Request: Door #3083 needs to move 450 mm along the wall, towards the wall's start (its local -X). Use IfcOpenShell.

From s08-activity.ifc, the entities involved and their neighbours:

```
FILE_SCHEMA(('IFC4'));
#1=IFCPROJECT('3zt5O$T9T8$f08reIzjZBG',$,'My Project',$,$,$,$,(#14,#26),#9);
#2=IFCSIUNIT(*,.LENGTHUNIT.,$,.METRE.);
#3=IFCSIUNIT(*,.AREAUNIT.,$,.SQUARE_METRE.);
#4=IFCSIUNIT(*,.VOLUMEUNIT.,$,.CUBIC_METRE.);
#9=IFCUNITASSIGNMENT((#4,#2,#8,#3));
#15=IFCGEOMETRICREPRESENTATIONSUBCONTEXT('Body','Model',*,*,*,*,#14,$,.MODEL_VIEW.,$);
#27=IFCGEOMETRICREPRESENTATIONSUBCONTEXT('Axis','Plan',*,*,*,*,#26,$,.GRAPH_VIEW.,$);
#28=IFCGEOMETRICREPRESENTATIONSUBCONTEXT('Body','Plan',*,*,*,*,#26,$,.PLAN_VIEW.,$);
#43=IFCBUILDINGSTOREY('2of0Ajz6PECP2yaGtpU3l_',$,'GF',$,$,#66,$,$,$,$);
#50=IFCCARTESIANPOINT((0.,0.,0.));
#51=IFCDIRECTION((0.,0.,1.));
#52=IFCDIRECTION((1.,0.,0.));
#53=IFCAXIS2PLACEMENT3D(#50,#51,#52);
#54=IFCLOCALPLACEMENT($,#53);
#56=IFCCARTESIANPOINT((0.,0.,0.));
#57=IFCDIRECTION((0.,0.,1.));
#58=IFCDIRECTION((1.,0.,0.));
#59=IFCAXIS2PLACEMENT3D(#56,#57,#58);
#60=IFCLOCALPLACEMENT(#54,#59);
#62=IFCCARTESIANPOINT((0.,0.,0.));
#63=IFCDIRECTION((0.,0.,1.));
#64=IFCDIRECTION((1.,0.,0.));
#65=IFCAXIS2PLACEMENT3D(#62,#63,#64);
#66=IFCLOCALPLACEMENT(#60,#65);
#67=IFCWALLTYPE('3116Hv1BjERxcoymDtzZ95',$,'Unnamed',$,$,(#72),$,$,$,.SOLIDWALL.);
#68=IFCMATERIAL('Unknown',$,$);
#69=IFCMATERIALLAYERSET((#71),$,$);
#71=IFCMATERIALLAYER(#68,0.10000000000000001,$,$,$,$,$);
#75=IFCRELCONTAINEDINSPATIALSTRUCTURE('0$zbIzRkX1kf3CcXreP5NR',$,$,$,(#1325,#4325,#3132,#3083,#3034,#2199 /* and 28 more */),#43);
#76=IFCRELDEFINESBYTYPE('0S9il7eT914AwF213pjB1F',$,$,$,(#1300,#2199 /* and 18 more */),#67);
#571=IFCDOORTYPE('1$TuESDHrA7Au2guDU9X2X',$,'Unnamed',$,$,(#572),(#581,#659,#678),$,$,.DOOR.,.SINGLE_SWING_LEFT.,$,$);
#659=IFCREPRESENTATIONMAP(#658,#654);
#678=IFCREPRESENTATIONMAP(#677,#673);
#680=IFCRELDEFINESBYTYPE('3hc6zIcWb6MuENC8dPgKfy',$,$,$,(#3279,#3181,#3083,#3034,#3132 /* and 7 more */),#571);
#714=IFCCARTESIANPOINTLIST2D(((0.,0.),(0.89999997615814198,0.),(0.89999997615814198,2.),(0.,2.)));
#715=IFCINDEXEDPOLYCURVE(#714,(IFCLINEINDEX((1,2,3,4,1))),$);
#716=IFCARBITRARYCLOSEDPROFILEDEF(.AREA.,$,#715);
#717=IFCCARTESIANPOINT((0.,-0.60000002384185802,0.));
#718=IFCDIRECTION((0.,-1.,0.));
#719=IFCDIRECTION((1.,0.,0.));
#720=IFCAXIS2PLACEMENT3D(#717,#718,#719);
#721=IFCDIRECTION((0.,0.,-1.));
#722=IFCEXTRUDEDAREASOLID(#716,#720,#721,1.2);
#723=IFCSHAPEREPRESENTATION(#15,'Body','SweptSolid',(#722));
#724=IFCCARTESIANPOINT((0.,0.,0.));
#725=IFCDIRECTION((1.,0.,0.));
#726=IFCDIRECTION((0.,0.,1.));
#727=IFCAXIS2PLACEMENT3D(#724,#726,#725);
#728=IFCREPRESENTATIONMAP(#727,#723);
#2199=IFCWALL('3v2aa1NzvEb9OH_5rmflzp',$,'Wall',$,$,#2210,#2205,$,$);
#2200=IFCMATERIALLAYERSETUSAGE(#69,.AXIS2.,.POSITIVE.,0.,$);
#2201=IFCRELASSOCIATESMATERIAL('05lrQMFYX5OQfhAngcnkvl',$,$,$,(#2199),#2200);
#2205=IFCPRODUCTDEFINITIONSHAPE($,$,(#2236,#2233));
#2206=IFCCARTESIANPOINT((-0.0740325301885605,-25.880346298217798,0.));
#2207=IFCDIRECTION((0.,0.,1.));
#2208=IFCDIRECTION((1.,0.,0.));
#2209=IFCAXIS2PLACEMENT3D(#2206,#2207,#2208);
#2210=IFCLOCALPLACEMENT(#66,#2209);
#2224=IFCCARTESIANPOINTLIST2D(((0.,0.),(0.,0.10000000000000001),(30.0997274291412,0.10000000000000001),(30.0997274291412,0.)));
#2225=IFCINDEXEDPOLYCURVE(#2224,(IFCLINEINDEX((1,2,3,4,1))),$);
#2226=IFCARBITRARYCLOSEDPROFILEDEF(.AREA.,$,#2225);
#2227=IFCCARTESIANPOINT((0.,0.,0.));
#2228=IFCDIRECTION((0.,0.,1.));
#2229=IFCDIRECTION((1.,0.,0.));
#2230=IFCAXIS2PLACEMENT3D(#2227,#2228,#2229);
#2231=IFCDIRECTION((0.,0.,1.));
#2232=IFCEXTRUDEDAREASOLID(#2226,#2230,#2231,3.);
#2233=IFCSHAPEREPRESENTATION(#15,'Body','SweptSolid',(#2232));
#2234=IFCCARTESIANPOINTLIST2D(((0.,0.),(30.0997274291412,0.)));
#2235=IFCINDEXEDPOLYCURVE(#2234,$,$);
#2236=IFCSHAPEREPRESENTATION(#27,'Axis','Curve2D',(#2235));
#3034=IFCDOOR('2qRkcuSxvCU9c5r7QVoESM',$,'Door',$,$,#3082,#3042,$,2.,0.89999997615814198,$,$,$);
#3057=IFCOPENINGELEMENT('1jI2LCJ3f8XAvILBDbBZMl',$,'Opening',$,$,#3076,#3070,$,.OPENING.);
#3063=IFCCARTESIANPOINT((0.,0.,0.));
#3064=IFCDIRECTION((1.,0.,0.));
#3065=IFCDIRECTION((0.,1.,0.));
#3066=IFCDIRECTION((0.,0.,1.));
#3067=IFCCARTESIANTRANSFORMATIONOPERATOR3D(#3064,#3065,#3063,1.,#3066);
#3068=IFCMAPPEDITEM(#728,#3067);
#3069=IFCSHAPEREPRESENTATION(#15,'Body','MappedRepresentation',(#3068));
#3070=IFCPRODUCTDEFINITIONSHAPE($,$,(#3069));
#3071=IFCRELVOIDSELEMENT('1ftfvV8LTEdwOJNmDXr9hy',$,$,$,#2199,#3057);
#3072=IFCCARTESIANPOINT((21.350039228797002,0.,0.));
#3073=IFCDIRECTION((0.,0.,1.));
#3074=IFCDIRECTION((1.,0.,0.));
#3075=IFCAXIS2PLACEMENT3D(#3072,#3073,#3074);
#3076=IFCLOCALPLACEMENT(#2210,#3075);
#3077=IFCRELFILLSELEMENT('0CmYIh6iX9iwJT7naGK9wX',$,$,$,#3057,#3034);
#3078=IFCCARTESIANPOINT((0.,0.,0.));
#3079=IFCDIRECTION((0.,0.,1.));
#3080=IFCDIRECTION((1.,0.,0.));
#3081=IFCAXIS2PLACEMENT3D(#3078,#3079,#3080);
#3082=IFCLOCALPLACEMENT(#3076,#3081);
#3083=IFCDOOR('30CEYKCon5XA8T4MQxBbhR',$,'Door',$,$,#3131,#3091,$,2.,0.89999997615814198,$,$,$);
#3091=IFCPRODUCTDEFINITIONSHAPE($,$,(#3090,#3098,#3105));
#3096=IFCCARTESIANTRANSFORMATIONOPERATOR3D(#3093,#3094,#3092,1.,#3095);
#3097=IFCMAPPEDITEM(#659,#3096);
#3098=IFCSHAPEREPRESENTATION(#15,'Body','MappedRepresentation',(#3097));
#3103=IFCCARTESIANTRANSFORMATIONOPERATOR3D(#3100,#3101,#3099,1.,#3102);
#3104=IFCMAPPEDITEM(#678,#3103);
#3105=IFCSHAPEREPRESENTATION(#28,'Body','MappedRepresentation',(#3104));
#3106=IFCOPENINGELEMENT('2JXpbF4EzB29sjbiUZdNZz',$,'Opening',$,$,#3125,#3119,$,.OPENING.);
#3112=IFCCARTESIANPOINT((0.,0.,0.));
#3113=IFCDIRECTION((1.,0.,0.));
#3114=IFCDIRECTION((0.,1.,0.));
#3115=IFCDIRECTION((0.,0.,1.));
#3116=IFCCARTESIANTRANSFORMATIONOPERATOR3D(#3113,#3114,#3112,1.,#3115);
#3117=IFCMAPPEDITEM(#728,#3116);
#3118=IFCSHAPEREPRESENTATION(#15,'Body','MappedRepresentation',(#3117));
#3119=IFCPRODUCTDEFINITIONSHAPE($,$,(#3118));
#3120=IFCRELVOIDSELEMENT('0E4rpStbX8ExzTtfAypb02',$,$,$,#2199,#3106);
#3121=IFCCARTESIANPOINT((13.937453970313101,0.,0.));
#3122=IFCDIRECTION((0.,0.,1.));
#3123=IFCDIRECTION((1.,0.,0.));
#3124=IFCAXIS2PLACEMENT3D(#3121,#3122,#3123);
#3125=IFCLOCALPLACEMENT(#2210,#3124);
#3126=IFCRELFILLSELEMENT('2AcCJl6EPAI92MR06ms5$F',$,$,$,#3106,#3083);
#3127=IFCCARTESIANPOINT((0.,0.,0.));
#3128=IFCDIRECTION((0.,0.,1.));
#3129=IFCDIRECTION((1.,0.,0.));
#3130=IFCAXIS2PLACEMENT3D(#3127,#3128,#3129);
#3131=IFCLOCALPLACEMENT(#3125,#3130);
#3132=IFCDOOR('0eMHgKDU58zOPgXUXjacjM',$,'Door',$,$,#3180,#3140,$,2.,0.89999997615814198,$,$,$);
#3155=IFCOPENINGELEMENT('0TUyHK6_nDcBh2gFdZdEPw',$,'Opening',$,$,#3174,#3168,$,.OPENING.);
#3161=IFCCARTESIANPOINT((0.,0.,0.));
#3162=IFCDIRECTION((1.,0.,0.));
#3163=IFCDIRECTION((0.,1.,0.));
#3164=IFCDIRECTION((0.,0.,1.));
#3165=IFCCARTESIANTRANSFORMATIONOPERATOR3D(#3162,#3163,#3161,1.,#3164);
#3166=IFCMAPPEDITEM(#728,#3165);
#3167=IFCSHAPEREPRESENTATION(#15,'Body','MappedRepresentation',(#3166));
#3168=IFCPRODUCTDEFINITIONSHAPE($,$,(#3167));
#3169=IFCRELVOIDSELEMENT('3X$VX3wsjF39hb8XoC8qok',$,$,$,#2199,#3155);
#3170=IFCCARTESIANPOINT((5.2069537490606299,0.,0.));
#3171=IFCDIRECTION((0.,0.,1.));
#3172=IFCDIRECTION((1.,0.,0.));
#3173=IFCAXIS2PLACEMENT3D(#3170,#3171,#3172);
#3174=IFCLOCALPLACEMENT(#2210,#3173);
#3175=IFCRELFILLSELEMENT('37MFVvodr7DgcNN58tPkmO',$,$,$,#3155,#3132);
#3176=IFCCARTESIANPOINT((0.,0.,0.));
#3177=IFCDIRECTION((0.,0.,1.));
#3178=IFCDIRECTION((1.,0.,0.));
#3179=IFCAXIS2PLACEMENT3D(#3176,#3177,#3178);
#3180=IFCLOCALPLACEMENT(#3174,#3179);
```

```python
import ifcopenshell
import ifcopenshell.api.geometry
import ifcopenshell.util.placement

model = ifcopenshell.open("s08-activity.ifc")

door = model.by_id(3083)
opening = door.FillsVoids[0].RelatingOpeningElement
wall = opening.VoidsElements[0].RelatingBuildingElement

wall_matrix = ifcopenshell.util.placement.get_local_placement(wall.ObjectPlacement)
shift = wall_matrix[:3, 0] * -0.45
before = ifcopenshell.util.placement.get_local_placement(door.ObjectPlacement)[:3, 3].copy()

# The door is placed relative to its opening, so it follows when the opening moves.
matrix = ifcopenshell.util.placement.get_local_placement(opening.ObjectPlacement)
matrix[:3, 3] += shift
ifcopenshell.api.geometry.edit_object_placement(
    model, product=opening, matrix=matrix, is_si=False, should_transform_children=True
)

after = ifcopenshell.util.placement.get_local_placement(door.ObjectPlacement)[:3, 3]
print("door moved by", (after - before).round(3) + 0.0)

model.write("s08-activity_updated.ifc")
```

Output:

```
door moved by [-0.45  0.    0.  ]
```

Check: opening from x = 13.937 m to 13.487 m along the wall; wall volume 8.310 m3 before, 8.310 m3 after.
